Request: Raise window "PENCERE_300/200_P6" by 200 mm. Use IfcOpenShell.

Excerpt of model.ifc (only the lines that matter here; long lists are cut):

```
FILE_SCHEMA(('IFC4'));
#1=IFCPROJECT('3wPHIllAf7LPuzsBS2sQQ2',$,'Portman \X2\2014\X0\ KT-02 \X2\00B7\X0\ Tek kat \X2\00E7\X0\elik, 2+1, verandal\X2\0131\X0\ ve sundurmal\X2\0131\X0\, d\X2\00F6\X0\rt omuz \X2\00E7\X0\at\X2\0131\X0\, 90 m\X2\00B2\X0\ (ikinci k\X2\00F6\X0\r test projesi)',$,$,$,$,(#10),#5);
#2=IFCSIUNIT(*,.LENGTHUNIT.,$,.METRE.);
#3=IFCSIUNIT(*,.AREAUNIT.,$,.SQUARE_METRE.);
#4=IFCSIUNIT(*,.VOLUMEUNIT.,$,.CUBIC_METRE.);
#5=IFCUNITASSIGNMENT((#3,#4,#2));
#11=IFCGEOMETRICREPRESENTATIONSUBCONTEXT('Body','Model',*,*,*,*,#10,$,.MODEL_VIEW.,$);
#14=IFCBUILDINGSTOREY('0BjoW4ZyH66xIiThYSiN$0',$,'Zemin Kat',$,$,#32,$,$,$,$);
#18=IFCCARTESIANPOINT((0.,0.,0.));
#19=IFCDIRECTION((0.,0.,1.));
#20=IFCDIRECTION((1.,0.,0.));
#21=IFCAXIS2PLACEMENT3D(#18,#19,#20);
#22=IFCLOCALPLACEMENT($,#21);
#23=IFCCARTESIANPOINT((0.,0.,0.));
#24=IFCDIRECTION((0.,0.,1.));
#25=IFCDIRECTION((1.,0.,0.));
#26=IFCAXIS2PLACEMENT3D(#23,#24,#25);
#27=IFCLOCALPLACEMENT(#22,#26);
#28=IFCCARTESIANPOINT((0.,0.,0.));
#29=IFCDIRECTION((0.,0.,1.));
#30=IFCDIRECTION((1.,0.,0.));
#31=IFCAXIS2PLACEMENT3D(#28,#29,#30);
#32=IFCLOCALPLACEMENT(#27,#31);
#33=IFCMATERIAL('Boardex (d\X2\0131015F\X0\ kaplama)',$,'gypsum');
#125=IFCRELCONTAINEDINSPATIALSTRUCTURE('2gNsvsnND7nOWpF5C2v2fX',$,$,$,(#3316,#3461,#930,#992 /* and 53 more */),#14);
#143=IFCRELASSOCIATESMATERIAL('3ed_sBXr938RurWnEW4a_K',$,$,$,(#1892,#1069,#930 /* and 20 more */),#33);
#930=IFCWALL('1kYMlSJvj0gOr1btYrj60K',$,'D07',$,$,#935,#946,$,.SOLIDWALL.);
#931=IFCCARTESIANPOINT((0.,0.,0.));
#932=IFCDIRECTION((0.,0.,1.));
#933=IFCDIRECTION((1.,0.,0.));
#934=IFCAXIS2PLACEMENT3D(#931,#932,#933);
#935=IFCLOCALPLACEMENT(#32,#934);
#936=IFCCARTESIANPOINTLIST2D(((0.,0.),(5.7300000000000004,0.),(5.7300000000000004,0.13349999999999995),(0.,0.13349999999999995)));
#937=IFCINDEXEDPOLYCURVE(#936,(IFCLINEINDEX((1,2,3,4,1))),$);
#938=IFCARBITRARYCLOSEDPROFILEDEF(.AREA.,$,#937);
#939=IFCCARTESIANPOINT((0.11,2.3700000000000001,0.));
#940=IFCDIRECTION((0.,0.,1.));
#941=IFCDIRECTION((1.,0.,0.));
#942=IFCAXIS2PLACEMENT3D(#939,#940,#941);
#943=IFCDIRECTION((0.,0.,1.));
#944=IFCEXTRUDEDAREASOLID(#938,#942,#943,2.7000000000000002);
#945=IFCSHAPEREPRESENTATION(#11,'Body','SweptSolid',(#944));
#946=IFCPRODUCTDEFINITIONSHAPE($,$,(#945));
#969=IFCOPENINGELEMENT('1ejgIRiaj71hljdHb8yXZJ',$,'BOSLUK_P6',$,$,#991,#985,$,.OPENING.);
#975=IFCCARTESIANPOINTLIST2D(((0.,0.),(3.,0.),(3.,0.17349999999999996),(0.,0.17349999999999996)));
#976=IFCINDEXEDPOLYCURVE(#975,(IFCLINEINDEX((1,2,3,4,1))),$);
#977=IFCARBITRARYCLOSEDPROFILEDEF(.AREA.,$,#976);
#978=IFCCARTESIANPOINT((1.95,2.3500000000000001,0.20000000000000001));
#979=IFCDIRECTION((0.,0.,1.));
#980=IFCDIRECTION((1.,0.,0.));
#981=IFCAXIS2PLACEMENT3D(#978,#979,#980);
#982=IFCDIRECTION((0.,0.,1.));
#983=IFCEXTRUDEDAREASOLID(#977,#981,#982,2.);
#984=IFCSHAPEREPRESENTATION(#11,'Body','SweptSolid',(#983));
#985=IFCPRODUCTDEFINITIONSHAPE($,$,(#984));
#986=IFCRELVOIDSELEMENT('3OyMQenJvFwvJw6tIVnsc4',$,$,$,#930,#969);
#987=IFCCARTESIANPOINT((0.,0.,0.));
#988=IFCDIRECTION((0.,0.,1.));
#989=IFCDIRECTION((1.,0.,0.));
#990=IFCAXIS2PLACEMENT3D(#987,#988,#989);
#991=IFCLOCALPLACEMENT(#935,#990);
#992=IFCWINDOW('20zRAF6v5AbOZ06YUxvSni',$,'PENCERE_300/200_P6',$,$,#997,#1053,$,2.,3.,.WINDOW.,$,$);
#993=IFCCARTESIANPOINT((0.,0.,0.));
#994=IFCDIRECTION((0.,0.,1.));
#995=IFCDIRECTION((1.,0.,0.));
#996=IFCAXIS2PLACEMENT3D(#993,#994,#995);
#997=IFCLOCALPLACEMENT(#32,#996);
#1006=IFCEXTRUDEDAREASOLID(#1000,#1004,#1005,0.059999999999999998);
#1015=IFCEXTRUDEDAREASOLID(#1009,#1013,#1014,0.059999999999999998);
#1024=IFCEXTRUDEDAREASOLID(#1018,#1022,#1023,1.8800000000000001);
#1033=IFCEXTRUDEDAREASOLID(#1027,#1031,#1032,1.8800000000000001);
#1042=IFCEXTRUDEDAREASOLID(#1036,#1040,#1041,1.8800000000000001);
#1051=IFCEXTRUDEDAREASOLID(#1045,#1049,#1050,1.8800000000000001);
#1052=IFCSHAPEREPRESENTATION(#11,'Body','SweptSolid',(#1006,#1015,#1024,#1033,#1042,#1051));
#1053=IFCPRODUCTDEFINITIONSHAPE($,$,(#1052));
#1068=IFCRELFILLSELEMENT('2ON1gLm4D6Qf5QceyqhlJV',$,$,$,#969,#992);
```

```python
import numpy as np
import ifcopenshell
import ifcopenshell.api.geometry
import ifcopenshell.util.placement
import ifcopenshell.util.unit

model = ifcopenshell.open("model.ifc")
unit_scale = ifcopenshell.util.unit.calculate_unit_scale(model)

window = model.by_id(992)
opening = window.FillsVoids[0].RelatingOpeningElement
dz = 0.2 / unit_scale

shift = np.array([0.0, 0.0, dz])
# The window is not placed relative to its opening, so move both.
for product in (opening, window):
    matrix = ifcopenshell.util.placement.get_local_placement(product.ObjectPlacement)
    matrix[:3, 3] += shift
    ifcopenshell.api.geometry.edit_object_placement(model, product=product, matrix=matrix, is_si=False)

print(f"moved by {dz * unit_scale:+.3f} m")

model.write("model_updated.ifc")
```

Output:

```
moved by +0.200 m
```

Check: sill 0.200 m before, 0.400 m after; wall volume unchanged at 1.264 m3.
